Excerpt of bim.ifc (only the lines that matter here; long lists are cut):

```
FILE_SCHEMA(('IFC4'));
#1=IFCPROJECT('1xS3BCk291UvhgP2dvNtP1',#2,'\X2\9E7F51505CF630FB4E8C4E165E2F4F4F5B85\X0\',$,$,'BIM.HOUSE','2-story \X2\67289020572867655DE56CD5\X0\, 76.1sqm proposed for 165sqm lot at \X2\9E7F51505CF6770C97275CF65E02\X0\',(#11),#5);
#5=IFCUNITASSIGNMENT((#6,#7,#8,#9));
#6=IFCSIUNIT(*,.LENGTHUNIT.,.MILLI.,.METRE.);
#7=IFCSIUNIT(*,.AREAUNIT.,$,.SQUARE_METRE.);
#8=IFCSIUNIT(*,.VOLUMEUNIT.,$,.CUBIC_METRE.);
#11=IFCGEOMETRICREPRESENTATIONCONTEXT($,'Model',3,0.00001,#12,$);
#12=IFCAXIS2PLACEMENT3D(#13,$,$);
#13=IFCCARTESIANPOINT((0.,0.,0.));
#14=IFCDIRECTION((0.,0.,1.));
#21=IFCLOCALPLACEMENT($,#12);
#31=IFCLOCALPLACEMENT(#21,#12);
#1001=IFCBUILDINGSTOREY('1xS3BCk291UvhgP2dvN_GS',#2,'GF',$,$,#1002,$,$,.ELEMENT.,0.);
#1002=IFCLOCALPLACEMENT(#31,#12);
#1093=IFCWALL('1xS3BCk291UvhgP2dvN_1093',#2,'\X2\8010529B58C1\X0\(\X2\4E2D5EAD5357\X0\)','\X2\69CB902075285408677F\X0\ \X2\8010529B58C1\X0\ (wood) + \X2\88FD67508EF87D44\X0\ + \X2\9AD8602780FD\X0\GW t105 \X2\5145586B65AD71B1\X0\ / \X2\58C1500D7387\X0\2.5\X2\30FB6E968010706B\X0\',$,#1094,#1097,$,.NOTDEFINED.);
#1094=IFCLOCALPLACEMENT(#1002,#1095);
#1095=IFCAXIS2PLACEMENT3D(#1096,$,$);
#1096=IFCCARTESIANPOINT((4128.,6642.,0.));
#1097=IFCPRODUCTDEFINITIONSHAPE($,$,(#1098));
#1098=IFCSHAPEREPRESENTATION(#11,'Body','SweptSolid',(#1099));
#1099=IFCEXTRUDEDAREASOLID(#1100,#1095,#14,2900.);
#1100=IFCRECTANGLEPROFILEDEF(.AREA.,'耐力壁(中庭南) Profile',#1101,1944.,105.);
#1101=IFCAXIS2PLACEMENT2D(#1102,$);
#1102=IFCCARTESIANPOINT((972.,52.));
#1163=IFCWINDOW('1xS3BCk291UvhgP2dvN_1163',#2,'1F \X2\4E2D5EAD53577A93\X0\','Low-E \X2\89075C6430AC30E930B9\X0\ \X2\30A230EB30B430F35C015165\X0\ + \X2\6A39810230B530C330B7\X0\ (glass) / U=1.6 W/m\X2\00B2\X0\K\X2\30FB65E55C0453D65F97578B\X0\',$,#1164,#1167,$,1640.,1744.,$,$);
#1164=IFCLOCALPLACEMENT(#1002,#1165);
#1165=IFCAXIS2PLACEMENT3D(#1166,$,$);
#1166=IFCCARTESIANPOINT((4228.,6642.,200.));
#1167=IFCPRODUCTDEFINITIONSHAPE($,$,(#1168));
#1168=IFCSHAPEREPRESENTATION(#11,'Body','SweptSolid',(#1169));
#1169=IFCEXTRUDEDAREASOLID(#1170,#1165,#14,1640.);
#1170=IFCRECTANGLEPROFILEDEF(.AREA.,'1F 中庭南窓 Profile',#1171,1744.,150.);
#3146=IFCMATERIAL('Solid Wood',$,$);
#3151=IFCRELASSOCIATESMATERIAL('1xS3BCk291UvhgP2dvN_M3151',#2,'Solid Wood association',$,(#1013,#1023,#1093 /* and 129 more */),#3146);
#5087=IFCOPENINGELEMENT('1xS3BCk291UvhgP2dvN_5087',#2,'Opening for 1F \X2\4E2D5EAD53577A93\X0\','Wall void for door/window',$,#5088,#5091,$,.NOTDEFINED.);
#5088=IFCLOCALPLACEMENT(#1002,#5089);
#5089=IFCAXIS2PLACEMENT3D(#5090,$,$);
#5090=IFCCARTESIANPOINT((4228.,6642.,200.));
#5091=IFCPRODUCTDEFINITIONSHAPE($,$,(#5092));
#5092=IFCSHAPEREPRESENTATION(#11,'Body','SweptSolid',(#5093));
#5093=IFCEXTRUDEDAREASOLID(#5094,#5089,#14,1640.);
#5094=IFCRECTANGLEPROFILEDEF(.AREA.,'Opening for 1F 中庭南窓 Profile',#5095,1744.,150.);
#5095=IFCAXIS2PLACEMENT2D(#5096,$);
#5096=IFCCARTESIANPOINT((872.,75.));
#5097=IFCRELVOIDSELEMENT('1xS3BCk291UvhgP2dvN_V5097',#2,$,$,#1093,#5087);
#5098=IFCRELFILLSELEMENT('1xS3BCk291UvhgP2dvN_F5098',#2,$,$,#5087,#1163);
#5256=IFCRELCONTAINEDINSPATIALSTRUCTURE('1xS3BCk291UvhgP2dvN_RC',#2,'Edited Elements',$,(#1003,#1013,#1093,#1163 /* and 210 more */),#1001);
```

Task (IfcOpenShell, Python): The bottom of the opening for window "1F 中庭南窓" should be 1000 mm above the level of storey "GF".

```python
import numpy as np
import ifcopenshell
import ifcopenshell.api.geometry
import ifcopenshell.geom
import ifcopenshell.util.element
import ifcopenshell.util.placement
import ifcopenshell.util.shape
import ifcopenshell.util.unit

model = ifcopenshell.open("bim.ifc")
unit_scale = ifcopenshell.util.unit.calculate_unit_scale(model)

window = model.by_guid("1xS3BCk291UvhgP2dvN_1163")
opening = window.FillsVoids[0].RelatingOpeningElement
storey = ifcopenshell.util.element.get_container(window, ifc_class="IfcBuildingStorey")
level = ifcopenshell.util.placement.get_local_placement(storey.ObjectPlacement)[2, 3]

# The opening's origin need not be at the sill, so measure its lowest point.
shape = ifcopenshell.geom.create_shape(ifcopenshell.geom.settings(), opening)
bottom = ifcopenshell.util.shape.get_shape_bottom_elevation(shape, shape.geometry) / unit_scale
dz = level + 1000.0 - bottom

shift = np.array([0.0, 0.0, dz])
# The window is not placed relative to its opening, so move both.
for product in (opening, window):
    matrix = ifcopenshell.util.placement.get_local_placement(product.ObjectPlacement)
    matrix[:3, 3] += shift
    ifcopenshell.api.geometry.edit_object_placement(model, product=product, matrix=matrix, is_si=False)

print(f"moved by {dz * unit_scale:+.3f} m")

model.write("bim_v2.ifc")
```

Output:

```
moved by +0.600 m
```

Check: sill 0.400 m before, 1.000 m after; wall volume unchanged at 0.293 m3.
